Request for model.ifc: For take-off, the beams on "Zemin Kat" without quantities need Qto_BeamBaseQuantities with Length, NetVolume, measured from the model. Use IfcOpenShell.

First a look at what the model holds.

```python
import ifcopenshell
import ifcopenshell.util.element
import ifcopenshell.util.unit

model = ifcopenshell.open("model.ifc")
print(model.schema)
for unit_type in ("LENGTHUNIT", "AREAUNIT", "VOLUMEUNIT"):
    print(unit_type, ifcopenshell.util.unit.calculate_unit_scale(model, unit_type))
storey = next(s for s in model.by_type("IfcBuildingStorey") if s.Name == "Zemin Kat")
beams = [e for e in ifcopenshell.util.element.get_decomposition(storey) if e.is_a("IfcBeam")]
for e in sorted(beams, key=lambda e: e.id()):
    print(e.id(), e.is_a(), e.Name, list(ifcopenshell.util.element.get_psets(e, qtos_only=True)), sep=" | ")
```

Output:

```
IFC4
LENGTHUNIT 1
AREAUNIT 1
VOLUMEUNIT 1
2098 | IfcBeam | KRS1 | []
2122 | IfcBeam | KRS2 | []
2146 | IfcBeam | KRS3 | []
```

```python
import ifcopenshell
import ifcopenshell.api.pset
import ifcopenshell.geom
import ifcopenshell.util.element
import ifcopenshell.util.shape
import ifcopenshell.util.unit

model = ifcopenshell.open("model.ifc")
unit_scale = ifcopenshell.util.unit.calculate_unit_scale(model)
volume_scale = ifcopenshell.util.unit.calculate_unit_scale(model, "VOLUMEUNIT")
settings = ifcopenshell.geom.settings()

storey = next(s for s in model.by_type("IfcBuildingStorey") if s.Name == "Zemin Kat")
beams = [e for e in ifcopenshell.util.element.get_decomposition(storey) if e.is_a("IfcBeam")]

for e in sorted(beams, key=lambda e: e.id()):
    if ifcopenshell.util.element.get_psets(e, qtos_only=True, should_inherit=False):
        continue
    # Geometry comes back in metres, in the element's own axes.
    shape = ifcopenshell.geom.create_shape(settings, e)
    values = {
        "Length": ifcopenshell.util.shape.get_max_xyz(shape.geometry) / unit_scale,
        "NetVolume": ifcopenshell.util.shape.get_volume(shape.geometry) / volume_scale,
    }
    qto = ifcopenshell.api.pset.add_qto(model, product=e, name="Qto_BeamBaseQuantities")
    ifcopenshell.api.pset.edit_qto(model, qto=qto, properties=values)
    print(e.id(), {k: round(v, 3) for k, v in values.items()})

model.write("model_v2.ifc")
```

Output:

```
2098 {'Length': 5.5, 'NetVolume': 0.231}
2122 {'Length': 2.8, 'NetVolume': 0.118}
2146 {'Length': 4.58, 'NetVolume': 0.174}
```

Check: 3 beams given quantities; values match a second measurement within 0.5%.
